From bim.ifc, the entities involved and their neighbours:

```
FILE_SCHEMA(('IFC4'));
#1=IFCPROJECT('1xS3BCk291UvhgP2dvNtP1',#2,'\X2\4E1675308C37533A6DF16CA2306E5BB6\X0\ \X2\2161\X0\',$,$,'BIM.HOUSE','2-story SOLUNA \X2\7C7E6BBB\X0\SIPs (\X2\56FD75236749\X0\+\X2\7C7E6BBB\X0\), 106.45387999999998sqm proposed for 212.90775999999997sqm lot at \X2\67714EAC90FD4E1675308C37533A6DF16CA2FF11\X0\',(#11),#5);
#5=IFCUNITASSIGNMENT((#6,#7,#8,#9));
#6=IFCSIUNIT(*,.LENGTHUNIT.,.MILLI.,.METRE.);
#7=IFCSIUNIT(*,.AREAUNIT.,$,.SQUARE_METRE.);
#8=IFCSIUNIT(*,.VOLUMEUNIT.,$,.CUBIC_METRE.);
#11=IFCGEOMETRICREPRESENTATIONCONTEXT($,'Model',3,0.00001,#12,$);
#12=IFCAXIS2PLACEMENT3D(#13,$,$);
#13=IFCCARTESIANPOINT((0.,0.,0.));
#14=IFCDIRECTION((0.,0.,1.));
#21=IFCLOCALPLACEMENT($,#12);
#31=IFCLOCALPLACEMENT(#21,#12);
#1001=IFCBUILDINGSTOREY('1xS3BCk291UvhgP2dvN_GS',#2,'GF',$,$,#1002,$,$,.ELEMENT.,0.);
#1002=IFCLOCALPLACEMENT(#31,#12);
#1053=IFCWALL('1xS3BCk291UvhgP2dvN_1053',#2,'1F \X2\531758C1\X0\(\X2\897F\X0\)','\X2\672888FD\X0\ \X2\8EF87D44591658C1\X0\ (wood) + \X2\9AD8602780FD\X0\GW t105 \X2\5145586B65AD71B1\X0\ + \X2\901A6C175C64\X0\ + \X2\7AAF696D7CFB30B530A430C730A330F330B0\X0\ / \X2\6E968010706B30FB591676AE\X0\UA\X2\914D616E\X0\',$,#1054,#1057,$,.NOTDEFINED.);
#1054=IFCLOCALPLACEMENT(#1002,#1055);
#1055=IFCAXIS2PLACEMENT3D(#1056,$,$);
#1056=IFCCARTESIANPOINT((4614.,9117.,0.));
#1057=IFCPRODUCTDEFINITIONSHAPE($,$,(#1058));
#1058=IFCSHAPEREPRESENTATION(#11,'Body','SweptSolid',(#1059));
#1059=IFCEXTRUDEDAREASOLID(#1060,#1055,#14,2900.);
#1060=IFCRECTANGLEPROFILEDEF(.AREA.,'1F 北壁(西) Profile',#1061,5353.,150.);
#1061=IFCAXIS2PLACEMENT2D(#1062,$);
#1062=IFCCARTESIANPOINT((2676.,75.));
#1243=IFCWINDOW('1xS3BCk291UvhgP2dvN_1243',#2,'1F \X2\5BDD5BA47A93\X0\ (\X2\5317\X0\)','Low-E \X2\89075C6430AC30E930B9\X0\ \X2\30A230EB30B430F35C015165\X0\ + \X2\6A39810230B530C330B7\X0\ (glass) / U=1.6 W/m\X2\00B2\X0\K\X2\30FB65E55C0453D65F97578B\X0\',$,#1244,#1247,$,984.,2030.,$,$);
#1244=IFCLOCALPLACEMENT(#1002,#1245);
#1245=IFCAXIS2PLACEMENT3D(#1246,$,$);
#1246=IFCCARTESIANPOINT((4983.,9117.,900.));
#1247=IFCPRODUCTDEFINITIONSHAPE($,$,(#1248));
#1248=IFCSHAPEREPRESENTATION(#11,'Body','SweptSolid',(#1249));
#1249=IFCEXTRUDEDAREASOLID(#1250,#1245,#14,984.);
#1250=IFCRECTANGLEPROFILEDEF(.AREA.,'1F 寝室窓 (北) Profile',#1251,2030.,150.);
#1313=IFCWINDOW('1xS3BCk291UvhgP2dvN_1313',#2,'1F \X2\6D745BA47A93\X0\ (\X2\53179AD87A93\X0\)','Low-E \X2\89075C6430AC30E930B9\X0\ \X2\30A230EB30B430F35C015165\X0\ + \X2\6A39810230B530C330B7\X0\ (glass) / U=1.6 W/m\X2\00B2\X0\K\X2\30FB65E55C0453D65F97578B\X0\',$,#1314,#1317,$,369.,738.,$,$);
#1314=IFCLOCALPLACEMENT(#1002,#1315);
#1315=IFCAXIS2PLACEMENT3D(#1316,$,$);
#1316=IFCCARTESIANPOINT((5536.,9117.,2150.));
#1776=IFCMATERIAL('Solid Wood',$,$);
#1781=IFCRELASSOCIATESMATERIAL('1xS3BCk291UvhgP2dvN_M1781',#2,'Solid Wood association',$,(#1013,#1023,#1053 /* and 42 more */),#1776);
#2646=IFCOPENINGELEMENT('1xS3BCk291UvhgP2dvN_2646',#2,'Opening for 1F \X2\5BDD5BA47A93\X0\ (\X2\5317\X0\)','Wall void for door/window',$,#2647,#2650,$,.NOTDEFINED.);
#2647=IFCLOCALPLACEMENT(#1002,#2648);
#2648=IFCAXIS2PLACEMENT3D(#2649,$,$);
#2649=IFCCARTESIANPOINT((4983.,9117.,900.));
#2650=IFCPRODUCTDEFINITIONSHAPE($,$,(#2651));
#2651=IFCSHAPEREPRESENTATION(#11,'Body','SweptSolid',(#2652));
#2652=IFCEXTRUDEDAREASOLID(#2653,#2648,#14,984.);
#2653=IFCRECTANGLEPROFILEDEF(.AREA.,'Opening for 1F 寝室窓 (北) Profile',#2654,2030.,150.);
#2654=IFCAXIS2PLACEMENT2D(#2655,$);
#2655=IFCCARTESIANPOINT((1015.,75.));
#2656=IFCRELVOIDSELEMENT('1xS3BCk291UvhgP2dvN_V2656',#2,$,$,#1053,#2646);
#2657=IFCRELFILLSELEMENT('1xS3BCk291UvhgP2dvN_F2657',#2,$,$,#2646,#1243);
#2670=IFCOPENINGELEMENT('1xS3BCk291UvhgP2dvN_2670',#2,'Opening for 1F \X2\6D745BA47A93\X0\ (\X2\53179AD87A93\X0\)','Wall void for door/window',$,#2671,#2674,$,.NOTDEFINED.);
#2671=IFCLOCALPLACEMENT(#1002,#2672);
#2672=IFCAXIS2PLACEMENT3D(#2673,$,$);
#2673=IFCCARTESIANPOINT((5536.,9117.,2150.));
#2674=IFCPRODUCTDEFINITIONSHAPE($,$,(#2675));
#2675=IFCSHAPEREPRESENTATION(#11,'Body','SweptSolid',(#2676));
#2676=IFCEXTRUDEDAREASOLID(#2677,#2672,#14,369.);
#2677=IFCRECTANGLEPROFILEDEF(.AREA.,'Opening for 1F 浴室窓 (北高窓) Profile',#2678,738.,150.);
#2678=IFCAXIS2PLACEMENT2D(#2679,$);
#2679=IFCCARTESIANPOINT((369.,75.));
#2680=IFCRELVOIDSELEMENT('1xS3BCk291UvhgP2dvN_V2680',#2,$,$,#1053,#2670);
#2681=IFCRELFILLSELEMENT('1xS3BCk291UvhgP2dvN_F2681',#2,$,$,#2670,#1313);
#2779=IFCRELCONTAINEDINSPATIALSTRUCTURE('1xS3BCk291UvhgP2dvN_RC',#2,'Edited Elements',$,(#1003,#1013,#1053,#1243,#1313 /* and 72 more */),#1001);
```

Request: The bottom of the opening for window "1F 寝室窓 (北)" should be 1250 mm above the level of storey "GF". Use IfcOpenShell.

```python
import numpy as np
import ifcopenshell
import ifcopenshell.api.geometry
import ifcopenshell.geom
import ifcopenshell.util.element
import ifcopenshell.util.placement
import ifcopenshell.util.shape
import ifcopenshell.util.unit

model = ifcopenshell.open("bim.ifc")
unit_scale = ifcopenshell.util.unit.calculate_unit_scale(model)

window = model.by_guid("1xS3BCk291UvhgP2dvN_1243")
opening = window.FillsVoids[0].RelatingOpeningElement
storey = ifcopenshell.util.element.get_container(window, ifc_class="IfcBuildingStorey")
level = ifcopenshell.util.placement.get_local_placement(storey.ObjectPlacement)[2, 3]

# The opening's origin need not be at the sill, so measure its lowest point.
shape = ifcopenshell.geom.create_shape(ifcopenshell.geom.settings(), opening)
bottom = ifcopenshell.util.shape.get_shape_bottom_elevation(shape, shape.geometry) / unit_scale
dz = level + 1.25 / unit_scale - bottom

shift = np.array([0.0, 0.0, dz])
# The window is not placed relative to its opening, so move both.
for product in (opening, window):
    matrix = ifcopenshell.util.placement.get_local_placement(product.ObjectPlacement)
    matrix[:3, 3] += shift
    ifcopenshell.api.geometry.edit_object_placement(model, product=product, matrix=matrix, is_si=False)

print(f"moved by {dz * unit_scale:+.3f} m")

model.write("bim_edited.ifc")
```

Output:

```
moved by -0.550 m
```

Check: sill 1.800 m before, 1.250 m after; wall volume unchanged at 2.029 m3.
